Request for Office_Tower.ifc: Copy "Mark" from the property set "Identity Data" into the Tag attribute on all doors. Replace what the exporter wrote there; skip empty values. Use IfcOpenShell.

First a look at what the model holds.

```python
import ifcopenshell
import ifcopenshell.util.element

model = ifcopenshell.open("Office_Tower.ifc")
print(model.schema)
doors = model.by_type("IfcDoor")
print(len(doors), "doors")
for e in doors[:8]:
    source = ifcopenshell.util.element.get_pset(e, "Identity Data", "Mark")
    target = e.Tag
    print(e.id(), repr(source), repr(target), sep=" | ")
```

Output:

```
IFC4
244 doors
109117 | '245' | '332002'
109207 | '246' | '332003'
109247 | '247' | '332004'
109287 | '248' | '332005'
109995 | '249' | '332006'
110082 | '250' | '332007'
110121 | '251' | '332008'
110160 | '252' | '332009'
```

```python
import ifcopenshell
import ifcopenshell.util.element

model = ifcopenshell.open("Office_Tower.ifc")

count = 0
for e in model.by_type("IfcDoor"):
    value = ifcopenshell.util.element.get_pset(e, "Identity Data", "Mark")
    current = e.Tag
    if not value or not value.strip() or current == value:
        continue
    e.Tag = value
    count += 1

print(count, "doors updated")

model.write("Office_Tower_rev.ifc")
```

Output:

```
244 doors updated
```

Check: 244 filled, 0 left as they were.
